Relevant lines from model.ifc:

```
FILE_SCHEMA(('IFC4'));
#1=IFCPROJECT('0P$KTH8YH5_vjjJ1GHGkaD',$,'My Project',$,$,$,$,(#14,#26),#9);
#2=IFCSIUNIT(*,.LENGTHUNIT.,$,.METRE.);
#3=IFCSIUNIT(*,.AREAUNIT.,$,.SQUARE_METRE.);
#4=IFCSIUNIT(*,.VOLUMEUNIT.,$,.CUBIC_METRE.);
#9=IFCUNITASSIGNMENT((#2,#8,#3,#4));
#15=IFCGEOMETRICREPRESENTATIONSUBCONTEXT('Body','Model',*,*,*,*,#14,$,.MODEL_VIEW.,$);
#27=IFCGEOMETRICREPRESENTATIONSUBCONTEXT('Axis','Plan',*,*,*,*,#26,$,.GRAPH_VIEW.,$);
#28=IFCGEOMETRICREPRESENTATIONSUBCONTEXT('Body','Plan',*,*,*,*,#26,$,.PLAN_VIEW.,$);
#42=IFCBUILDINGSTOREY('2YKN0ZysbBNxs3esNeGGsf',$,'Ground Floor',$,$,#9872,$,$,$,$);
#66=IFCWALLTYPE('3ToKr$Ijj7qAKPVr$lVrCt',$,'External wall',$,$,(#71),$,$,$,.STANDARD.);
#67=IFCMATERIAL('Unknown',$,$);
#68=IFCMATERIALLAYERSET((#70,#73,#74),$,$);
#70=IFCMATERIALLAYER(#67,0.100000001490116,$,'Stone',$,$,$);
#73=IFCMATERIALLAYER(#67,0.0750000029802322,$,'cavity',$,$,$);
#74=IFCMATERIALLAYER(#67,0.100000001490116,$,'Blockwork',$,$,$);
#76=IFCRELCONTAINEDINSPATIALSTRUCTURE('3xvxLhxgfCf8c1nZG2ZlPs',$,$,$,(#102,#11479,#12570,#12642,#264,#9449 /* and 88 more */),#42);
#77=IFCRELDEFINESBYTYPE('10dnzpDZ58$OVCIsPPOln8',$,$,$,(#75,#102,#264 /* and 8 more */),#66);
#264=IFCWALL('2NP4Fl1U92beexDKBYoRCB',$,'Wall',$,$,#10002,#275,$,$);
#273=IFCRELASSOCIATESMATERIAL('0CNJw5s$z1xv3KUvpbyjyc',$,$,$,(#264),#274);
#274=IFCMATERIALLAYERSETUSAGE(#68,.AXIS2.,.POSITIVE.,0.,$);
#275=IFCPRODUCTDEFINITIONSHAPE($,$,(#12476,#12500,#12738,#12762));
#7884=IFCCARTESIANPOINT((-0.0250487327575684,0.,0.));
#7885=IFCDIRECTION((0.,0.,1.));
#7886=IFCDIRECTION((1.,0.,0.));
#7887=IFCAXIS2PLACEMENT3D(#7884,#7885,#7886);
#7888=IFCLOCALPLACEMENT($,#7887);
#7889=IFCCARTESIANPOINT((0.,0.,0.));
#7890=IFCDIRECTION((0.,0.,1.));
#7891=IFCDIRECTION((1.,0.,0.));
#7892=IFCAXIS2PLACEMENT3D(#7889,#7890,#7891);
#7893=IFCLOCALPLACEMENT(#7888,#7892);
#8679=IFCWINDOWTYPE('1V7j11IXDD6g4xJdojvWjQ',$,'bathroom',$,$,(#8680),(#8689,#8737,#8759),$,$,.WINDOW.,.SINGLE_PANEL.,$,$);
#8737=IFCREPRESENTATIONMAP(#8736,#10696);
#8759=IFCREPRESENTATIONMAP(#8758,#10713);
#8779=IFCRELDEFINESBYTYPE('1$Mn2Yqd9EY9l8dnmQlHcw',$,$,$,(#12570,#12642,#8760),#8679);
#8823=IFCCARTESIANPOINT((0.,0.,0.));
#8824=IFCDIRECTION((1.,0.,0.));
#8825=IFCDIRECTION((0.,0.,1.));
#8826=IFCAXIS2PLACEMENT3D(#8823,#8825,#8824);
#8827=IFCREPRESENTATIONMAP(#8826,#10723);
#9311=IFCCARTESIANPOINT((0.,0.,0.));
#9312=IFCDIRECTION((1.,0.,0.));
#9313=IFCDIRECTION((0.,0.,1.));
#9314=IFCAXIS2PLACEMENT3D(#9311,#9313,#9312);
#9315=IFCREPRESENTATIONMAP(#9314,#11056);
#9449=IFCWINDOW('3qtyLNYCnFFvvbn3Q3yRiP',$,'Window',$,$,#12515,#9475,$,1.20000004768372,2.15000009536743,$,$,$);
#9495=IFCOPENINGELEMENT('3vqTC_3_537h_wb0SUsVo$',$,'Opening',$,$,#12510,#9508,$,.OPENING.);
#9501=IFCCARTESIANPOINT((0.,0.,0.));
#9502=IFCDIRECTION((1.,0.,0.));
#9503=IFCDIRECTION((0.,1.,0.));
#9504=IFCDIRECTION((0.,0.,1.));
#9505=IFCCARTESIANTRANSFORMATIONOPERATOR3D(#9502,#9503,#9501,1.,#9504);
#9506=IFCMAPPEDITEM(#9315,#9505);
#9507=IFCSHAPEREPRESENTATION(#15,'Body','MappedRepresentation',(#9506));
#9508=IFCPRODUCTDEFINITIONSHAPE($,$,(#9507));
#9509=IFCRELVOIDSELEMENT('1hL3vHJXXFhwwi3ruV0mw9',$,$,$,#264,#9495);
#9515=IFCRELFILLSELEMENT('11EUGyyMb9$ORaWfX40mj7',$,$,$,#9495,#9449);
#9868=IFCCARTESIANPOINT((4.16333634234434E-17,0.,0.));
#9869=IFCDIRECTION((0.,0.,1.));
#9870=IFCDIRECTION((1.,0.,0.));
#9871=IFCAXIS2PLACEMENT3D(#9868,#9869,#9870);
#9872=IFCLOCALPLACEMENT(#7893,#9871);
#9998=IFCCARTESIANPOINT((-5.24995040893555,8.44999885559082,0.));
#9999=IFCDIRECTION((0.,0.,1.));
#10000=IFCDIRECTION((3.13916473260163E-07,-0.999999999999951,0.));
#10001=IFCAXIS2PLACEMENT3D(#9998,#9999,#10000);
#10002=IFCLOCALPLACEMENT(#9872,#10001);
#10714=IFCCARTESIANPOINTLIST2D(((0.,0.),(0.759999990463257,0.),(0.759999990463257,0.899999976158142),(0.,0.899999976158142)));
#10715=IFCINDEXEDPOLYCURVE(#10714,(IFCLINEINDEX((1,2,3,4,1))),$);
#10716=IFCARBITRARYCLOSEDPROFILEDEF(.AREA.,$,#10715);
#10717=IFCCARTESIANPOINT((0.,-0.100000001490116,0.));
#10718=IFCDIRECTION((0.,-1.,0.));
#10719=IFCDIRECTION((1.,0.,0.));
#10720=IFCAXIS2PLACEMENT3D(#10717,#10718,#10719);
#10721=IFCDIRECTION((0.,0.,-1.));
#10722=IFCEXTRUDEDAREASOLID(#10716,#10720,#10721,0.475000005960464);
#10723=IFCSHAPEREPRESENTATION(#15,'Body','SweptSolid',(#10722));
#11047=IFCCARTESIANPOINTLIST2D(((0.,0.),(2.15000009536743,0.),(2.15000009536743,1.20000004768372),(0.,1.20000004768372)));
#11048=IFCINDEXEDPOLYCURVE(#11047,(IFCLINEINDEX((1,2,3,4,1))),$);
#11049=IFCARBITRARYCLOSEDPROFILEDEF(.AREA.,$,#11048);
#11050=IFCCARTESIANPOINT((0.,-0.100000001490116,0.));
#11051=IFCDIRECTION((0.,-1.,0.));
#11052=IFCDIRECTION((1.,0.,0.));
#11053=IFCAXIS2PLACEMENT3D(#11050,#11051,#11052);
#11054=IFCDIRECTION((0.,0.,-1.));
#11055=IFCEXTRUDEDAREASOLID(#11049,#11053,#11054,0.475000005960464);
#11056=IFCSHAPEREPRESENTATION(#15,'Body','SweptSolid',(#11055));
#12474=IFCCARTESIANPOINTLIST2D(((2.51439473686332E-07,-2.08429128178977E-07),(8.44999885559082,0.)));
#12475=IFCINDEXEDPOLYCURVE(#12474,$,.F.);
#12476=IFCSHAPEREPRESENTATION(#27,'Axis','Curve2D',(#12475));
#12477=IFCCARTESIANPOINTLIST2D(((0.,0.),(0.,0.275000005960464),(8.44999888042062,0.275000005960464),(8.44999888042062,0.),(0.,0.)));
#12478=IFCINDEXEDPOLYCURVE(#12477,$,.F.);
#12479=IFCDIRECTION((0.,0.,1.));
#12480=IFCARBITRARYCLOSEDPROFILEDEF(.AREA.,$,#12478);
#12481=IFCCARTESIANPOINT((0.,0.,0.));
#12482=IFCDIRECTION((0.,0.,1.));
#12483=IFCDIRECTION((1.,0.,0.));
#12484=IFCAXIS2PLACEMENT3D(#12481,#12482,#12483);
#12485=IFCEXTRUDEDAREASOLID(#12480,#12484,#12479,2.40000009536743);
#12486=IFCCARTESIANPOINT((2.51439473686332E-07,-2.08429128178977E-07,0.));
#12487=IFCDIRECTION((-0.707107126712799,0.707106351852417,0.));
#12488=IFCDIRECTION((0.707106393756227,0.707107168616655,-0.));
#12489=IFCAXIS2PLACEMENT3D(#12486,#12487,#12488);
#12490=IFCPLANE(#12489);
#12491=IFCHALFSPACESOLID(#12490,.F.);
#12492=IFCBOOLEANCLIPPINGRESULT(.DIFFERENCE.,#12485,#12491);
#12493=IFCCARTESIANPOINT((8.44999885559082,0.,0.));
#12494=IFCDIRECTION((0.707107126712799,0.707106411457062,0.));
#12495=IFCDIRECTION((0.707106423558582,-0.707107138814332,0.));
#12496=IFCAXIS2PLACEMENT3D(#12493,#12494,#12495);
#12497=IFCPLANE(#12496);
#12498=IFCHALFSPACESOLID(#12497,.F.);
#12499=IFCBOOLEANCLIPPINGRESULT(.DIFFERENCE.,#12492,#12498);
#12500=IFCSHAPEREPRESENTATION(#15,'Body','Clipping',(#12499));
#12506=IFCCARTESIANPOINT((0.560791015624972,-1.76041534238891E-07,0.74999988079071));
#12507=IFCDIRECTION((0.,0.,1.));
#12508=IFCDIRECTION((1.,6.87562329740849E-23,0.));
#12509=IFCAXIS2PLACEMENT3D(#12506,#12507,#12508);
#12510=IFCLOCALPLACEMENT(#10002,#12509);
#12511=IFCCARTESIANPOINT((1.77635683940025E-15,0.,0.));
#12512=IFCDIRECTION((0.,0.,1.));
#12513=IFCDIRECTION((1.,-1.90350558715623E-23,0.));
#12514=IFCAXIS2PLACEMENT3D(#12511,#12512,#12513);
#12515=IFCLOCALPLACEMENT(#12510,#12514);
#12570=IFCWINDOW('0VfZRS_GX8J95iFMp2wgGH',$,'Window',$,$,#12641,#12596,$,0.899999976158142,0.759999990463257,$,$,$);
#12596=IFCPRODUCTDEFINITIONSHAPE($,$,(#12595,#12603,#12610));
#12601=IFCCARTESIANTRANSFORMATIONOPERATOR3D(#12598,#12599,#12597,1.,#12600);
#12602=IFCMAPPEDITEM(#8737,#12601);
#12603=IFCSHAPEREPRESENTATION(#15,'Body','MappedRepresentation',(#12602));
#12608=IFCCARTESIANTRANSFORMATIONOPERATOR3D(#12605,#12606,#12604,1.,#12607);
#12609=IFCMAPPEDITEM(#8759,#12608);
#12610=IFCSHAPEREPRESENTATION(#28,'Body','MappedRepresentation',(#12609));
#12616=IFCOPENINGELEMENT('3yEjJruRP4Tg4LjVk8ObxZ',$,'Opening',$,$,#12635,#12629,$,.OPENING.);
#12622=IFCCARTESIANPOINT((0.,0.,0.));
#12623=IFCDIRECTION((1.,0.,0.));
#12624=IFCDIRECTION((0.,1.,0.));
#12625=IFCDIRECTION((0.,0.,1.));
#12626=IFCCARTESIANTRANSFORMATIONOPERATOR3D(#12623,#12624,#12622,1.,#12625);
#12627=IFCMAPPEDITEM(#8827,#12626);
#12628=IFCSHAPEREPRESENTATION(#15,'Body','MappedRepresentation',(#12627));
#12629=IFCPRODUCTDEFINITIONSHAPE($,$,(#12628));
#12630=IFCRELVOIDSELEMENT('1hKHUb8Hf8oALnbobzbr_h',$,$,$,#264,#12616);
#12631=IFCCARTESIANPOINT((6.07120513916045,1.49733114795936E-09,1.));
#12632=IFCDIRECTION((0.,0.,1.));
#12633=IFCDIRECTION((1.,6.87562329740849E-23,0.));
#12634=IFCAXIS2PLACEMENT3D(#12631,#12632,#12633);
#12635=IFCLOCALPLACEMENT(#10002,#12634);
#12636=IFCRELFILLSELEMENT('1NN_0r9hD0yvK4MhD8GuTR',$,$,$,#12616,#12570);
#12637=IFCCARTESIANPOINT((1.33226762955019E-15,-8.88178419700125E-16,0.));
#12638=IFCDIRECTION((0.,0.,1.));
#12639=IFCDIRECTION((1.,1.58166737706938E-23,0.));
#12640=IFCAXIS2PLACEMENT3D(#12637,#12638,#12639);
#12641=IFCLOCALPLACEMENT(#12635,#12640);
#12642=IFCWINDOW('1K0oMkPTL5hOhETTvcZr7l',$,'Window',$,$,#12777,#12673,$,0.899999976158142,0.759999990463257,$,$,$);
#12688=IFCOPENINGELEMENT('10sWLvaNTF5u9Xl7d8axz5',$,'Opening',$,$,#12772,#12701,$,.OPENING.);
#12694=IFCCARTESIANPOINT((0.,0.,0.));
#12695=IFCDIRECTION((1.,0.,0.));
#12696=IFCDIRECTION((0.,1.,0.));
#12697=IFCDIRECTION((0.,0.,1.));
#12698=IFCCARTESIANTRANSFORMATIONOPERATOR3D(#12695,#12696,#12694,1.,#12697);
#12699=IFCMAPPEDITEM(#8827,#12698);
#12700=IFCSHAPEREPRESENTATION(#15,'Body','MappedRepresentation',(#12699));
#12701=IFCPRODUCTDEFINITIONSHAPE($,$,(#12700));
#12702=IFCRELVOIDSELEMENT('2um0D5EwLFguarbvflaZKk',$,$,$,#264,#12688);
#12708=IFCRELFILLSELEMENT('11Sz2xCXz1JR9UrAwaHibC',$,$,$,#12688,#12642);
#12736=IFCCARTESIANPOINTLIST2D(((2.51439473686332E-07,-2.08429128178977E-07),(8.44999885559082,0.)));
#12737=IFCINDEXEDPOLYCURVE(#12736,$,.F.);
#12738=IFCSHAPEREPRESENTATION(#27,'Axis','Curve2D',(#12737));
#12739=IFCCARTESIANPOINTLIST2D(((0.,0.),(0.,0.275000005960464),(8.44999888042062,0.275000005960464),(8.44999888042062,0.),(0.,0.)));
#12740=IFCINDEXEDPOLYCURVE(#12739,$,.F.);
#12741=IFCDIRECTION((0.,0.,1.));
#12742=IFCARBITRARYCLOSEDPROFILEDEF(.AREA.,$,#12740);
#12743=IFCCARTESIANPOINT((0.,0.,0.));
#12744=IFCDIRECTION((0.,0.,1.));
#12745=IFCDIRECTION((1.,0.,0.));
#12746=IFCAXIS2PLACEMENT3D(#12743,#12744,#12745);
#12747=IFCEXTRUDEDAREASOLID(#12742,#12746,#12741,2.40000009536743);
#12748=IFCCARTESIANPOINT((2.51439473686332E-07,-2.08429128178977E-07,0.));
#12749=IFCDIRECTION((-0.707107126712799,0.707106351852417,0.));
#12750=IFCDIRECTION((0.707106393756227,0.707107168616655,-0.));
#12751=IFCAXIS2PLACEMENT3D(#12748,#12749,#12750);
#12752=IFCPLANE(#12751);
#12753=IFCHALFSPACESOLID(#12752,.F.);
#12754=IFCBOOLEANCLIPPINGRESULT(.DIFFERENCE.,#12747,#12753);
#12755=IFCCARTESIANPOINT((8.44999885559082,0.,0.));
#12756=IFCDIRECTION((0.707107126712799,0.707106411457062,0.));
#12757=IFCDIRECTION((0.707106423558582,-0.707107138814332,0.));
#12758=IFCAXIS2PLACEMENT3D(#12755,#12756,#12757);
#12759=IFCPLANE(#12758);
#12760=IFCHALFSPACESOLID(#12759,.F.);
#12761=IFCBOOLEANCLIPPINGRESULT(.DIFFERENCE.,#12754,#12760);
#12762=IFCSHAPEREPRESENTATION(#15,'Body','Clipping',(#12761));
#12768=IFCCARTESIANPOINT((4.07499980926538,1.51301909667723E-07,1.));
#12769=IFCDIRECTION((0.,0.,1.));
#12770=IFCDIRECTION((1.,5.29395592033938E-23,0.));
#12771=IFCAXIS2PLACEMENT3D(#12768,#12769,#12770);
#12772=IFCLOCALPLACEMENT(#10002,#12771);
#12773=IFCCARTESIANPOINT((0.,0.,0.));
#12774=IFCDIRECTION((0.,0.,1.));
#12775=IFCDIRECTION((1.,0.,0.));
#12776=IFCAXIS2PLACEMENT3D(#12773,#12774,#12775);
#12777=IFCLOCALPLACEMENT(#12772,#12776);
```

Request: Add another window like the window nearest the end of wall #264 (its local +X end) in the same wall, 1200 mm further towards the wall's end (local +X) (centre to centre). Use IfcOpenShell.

```python
import ifcopenshell
import ifcopenshell.api.feature
import ifcopenshell.api.geometry
import ifcopenshell.api.root
import ifcopenshell.geom
import ifcopenshell.util.element
import ifcopenshell.util.placement
import ifcopenshell.util.shape
import ifcopenshell.util.unit

model = ifcopenshell.open("model.ifc")
unit_scale = ifcopenshell.util.unit.calculate_unit_scale(model)
settings = ifcopenshell.geom.settings()


def volume(element):
    """Net volume in cubic metres, openings subtracted."""
    shape = ifcopenshell.geom.create_shape(settings, element)
    return ifcopenshell.util.shape.get_volume(shape.geometry)


window = model.by_id(12570)
opening = window.FillsVoids[0].RelatingOpeningElement
wall = opening.VoidsElements[0].RelatingBuildingElement
before = volume(wall)
shift = ifcopenshell.util.placement.get_local_placement(wall.ObjectPlacement)[:3, 0] * 1.2 / unit_scale

# copy_class copies the void relationship, type, container and properties, but no geometry.
new_opening = ifcopenshell.api.root.copy_class(model, product=opening)
new_opening.Representation = ifcopenshell.util.element.copy_deep(
    model, opening.Representation, exclude=["IfcGeometricRepresentationContext", "IfcRepresentationMap"]
)
new_window = ifcopenshell.api.root.copy_class(model, product=window)
new_window.Representation = ifcopenshell.util.element.copy_deep(
    model, window.Representation, exclude=["IfcGeometricRepresentationContext", "IfcRepresentationMap"]
)
ifcopenshell.api.feature.add_filling(model, opening=new_opening, element=new_window)

for old, new in ((opening, new_opening), (window, new_window)):
    matrix = ifcopenshell.util.placement.get_local_placement(old.ObjectPlacement)
    matrix[:3, 3] += shift
    ifcopenshell.api.geometry.edit_object_placement(model, product=new, matrix=matrix, is_si=False)

after = volume(wall)

print(f"wall volume {before:.3f} -> {after:.3f} m3")

model.write("model_v2.ifc")
```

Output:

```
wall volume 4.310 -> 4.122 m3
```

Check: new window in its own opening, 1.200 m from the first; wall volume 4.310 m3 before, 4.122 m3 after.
